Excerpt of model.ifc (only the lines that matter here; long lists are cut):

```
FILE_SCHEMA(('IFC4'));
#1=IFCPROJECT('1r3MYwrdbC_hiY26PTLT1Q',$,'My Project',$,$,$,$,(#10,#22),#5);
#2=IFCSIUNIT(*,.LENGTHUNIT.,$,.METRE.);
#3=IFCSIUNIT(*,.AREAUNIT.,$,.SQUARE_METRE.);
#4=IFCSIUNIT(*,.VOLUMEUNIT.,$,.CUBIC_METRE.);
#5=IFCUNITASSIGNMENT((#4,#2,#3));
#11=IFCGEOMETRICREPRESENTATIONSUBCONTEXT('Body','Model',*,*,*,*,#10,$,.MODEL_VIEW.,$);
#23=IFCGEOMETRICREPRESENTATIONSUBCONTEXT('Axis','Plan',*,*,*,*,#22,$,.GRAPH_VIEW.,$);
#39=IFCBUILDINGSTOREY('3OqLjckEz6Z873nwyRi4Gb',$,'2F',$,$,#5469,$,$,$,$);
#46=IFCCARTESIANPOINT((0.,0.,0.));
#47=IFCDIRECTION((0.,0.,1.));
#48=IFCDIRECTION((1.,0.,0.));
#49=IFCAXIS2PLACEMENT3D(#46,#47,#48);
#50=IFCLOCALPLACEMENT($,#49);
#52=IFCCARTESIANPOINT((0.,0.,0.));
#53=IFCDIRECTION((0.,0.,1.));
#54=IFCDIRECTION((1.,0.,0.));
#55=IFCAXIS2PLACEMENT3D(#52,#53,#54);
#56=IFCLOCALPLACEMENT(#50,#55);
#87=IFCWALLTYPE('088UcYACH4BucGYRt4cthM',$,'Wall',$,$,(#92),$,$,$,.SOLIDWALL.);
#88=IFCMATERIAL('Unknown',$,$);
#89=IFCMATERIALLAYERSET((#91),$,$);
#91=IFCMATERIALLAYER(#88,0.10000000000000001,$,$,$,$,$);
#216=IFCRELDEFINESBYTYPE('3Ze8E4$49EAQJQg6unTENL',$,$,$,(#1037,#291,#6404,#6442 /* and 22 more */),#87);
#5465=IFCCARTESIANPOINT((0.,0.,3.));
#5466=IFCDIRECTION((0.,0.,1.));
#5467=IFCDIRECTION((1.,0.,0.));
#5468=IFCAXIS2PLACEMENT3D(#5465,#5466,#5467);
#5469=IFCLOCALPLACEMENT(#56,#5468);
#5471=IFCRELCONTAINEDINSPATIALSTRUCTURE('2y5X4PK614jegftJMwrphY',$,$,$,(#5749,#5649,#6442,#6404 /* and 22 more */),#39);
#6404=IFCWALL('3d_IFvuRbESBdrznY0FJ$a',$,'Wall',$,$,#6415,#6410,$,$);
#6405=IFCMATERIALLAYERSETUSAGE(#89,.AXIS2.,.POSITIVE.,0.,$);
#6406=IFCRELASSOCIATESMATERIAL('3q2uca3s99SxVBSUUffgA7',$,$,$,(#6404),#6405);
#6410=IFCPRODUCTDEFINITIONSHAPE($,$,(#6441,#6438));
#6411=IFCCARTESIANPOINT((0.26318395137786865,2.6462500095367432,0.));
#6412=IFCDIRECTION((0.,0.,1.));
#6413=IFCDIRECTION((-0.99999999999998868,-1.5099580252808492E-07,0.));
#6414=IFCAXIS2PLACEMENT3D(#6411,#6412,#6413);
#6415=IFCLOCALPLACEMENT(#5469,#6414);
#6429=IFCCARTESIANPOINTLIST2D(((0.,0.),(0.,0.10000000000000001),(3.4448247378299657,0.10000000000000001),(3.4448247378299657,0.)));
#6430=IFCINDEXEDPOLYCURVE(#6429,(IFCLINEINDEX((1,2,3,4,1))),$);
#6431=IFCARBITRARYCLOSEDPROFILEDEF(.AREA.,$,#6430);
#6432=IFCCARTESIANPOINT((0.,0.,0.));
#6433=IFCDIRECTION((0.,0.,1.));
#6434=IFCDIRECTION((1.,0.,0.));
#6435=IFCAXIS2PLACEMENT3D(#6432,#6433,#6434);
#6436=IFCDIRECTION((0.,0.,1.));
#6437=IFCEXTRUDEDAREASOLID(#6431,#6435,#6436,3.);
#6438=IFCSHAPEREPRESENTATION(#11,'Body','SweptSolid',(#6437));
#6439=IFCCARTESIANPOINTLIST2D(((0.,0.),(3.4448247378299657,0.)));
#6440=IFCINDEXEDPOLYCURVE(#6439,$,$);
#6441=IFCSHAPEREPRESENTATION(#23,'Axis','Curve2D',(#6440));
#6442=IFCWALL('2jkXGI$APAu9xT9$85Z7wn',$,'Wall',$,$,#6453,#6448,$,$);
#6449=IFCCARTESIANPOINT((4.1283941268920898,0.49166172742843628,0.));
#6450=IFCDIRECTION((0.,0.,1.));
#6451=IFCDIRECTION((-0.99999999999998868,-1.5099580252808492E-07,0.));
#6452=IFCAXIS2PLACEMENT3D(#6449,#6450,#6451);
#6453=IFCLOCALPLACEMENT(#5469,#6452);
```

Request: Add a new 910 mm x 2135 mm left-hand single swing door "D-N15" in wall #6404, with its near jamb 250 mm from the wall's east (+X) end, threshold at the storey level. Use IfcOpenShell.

```python
import numpy as np
import ifcopenshell
import ifcopenshell.api.feature
import ifcopenshell.api.geometry
import ifcopenshell.api.root
import ifcopenshell.api.spatial
import ifcopenshell.geom
import ifcopenshell.util.element
import ifcopenshell.util.placement
import ifcopenshell.util.representation
import ifcopenshell.util.shape
import ifcopenshell.util.unit

model = ifcopenshell.open("model.ifc")
unit_scale = ifcopenshell.util.unit.calculate_unit_scale(model)
settings = ifcopenshell.geom.settings()


def volume(element):
    """Net volume in cubic metres, openings subtracted."""
    shape = ifcopenshell.geom.create_shape(settings, element)
    return ifcopenshell.util.shape.get_volume(shape.geometry)


wall = model.by_id(6404)
storey = ifcopenshell.util.element.get_container(wall, ifc_class="IfcBuildingStorey")
context = ifcopenshell.util.representation.get_context(model, "Model", "Body", "MODEL_VIEW")
before = volume(wall)

width, height, from_end, sill = 0.91, 2.135, 0.25, 0.0  # metres

# The wall runs along its own X axis, and the end named is its -X end.
wall_shape = ifcopenshell.geom.create_shape(settings, wall)
x, y, z = ifcopenshell.util.shape.get_vertices(wall_shape.geometry).T
start = x.min() + from_end
face, thickness = float(y.min()), float(y.max() - y.min())
wall_matrix = ifcopenshell.util.placement.get_local_placement(wall.ObjectPlacement)
level = ifcopenshell.util.placement.get_local_placement(storey.ObjectPlacement)[2, 3]


def in_wall(x, y):
    """Placement at x, y metres in the wall's axes, at sill height."""
    matrix = wall_matrix.copy()
    matrix[:, 3] = wall_matrix @ np.array([x / unit_scale, y / unit_scale, 0.0, 1.0])
    matrix[2, 3] = level + sill / unit_scale
    return matrix


# Opening: a box that overshoots both wall faces by 50 mm.
opening = ifcopenshell.api.root.create_entity(model, ifc_class="IfcOpeningElement", predefined_type="OPENING")
box = ifcopenshell.api.geometry.add_wall_representation(
    model, context=context, length=width, height=height, thickness=thickness + 0.1
)
ifcopenshell.api.geometry.assign_representation(model, product=opening, representation=box)
ifcopenshell.api.geometry.edit_object_placement(model, product=opening, matrix=in_wall(start, face - 0.05), is_si=False)
ifcopenshell.api.feature.add_feature(model, feature=opening, element=wall)

door = ifcopenshell.api.root.create_entity(model, ifc_class="IfcDoor", name="D-N15", predefined_type="DOOR")
door.OverallWidth, door.OverallHeight = width / unit_scale, height / unit_scale
door.OperationType = "SINGLE_SWING_LEFT"
body = ifcopenshell.api.geometry.add_door_representation(
    model,
    context=context,
    overall_width=door.OverallWidth,
    overall_height=door.OverallHeight,
    operation_type="SINGLE_SWING_LEFT",
    lining_properties={"LiningDepth": thickness / unit_scale, "ThresholdDepth": thickness / unit_scale},
)
ifcopenshell.api.geometry.assign_representation(model, product=door, representation=body)
ifcopenshell.api.spatial.assign_container(model, products=[door], relating_structure=storey)
ifcopenshell.api.feature.add_filling(model, opening=opening, element=door)

# The lining spans the wall, so the door starts at the wall face.
ifcopenshell.api.geometry.edit_object_placement(model, product=door, matrix=in_wall(start, face), is_si=False)

after = volume(wall)

print(f"wall volume {before:.3f} -> {after:.3f} m3")

model.write("model_v2.ifc")
```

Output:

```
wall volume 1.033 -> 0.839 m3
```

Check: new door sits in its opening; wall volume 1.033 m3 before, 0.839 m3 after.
